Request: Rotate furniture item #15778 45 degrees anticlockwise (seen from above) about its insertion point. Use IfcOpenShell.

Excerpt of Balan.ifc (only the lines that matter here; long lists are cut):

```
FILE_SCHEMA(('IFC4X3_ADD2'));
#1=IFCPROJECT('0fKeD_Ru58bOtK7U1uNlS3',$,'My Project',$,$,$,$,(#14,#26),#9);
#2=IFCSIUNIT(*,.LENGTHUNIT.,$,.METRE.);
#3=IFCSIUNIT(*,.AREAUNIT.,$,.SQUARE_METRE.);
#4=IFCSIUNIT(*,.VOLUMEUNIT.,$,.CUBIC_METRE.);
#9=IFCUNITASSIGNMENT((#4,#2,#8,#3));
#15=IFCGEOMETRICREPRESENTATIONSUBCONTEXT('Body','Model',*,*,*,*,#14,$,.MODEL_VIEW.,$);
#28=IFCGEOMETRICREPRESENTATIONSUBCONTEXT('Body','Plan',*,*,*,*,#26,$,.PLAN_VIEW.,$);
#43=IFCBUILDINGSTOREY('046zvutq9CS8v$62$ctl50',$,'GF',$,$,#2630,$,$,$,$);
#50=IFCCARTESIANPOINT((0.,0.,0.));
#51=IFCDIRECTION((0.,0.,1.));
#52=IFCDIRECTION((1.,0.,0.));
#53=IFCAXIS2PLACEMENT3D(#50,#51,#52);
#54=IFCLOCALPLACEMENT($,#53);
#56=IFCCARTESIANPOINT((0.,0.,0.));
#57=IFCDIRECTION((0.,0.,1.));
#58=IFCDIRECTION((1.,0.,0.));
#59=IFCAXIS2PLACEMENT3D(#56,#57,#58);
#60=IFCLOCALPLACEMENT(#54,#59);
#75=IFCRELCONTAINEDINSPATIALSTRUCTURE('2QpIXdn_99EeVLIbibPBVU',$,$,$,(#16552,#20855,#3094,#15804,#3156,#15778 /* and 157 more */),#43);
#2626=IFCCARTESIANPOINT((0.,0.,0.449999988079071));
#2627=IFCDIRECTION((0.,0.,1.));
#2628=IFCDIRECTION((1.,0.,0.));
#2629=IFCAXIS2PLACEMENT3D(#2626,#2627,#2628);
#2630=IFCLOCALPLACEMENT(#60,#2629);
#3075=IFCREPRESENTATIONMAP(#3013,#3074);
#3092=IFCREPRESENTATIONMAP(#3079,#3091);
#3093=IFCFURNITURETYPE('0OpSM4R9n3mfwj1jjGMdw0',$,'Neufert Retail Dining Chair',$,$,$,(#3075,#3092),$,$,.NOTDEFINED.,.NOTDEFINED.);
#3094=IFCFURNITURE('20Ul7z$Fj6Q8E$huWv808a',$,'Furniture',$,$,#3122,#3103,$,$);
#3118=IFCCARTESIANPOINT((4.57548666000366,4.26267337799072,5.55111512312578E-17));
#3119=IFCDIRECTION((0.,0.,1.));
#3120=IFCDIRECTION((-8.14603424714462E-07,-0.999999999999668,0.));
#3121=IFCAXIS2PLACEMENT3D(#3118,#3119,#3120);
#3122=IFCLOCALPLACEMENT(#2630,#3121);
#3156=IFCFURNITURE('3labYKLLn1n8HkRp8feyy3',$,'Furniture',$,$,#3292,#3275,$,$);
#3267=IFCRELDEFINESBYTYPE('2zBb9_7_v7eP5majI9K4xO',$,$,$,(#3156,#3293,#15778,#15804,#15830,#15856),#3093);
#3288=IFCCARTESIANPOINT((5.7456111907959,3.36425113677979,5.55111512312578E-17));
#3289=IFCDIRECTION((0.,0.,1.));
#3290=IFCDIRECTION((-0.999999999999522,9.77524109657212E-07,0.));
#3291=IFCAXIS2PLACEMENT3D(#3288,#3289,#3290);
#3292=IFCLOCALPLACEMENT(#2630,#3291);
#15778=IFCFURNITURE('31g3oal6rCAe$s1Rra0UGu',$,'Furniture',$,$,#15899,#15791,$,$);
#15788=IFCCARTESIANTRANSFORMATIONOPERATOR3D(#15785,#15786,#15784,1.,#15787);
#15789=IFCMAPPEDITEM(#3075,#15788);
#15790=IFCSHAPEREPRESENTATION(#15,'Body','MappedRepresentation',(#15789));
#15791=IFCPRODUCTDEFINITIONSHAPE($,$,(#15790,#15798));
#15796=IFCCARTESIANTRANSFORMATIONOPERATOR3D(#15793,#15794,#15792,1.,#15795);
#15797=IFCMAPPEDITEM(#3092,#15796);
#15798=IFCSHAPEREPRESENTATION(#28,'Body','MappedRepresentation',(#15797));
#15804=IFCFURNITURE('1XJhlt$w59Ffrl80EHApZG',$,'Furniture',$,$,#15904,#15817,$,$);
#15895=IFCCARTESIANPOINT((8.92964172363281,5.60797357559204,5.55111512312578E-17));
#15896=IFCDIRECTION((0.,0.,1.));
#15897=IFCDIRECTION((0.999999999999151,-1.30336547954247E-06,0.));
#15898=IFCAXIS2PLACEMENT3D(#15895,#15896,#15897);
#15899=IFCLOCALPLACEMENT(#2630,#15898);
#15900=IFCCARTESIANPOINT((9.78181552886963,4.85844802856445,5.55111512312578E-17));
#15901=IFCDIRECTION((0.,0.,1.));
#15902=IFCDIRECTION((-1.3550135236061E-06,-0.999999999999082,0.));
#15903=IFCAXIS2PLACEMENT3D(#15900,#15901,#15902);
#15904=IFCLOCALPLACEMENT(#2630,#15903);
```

```python
import ifcopenshell
import ifcopenshell.api.geometry
import ifcopenshell.util.placement

model = ifcopenshell.open("Balan.ifc")

item = model.by_guid("31g3oal6rCAe$s1Rra0UGu")
matrix = ifcopenshell.util.placement.get_local_placement(item.ObjectPlacement)
matrix = matrix @ ifcopenshell.util.placement.rotation(45, "Z")
ifcopenshell.api.geometry.edit_object_placement(model, product=item, matrix=matrix, is_si=False)

print(ifcopenshell.util.placement.get_local_placement(item.ObjectPlacement).round(3) + 0.0)

model.write("Balan-out.ifc")
```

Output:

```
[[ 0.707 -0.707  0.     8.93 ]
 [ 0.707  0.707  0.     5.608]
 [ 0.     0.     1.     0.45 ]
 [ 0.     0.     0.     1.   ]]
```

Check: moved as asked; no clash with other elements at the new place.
